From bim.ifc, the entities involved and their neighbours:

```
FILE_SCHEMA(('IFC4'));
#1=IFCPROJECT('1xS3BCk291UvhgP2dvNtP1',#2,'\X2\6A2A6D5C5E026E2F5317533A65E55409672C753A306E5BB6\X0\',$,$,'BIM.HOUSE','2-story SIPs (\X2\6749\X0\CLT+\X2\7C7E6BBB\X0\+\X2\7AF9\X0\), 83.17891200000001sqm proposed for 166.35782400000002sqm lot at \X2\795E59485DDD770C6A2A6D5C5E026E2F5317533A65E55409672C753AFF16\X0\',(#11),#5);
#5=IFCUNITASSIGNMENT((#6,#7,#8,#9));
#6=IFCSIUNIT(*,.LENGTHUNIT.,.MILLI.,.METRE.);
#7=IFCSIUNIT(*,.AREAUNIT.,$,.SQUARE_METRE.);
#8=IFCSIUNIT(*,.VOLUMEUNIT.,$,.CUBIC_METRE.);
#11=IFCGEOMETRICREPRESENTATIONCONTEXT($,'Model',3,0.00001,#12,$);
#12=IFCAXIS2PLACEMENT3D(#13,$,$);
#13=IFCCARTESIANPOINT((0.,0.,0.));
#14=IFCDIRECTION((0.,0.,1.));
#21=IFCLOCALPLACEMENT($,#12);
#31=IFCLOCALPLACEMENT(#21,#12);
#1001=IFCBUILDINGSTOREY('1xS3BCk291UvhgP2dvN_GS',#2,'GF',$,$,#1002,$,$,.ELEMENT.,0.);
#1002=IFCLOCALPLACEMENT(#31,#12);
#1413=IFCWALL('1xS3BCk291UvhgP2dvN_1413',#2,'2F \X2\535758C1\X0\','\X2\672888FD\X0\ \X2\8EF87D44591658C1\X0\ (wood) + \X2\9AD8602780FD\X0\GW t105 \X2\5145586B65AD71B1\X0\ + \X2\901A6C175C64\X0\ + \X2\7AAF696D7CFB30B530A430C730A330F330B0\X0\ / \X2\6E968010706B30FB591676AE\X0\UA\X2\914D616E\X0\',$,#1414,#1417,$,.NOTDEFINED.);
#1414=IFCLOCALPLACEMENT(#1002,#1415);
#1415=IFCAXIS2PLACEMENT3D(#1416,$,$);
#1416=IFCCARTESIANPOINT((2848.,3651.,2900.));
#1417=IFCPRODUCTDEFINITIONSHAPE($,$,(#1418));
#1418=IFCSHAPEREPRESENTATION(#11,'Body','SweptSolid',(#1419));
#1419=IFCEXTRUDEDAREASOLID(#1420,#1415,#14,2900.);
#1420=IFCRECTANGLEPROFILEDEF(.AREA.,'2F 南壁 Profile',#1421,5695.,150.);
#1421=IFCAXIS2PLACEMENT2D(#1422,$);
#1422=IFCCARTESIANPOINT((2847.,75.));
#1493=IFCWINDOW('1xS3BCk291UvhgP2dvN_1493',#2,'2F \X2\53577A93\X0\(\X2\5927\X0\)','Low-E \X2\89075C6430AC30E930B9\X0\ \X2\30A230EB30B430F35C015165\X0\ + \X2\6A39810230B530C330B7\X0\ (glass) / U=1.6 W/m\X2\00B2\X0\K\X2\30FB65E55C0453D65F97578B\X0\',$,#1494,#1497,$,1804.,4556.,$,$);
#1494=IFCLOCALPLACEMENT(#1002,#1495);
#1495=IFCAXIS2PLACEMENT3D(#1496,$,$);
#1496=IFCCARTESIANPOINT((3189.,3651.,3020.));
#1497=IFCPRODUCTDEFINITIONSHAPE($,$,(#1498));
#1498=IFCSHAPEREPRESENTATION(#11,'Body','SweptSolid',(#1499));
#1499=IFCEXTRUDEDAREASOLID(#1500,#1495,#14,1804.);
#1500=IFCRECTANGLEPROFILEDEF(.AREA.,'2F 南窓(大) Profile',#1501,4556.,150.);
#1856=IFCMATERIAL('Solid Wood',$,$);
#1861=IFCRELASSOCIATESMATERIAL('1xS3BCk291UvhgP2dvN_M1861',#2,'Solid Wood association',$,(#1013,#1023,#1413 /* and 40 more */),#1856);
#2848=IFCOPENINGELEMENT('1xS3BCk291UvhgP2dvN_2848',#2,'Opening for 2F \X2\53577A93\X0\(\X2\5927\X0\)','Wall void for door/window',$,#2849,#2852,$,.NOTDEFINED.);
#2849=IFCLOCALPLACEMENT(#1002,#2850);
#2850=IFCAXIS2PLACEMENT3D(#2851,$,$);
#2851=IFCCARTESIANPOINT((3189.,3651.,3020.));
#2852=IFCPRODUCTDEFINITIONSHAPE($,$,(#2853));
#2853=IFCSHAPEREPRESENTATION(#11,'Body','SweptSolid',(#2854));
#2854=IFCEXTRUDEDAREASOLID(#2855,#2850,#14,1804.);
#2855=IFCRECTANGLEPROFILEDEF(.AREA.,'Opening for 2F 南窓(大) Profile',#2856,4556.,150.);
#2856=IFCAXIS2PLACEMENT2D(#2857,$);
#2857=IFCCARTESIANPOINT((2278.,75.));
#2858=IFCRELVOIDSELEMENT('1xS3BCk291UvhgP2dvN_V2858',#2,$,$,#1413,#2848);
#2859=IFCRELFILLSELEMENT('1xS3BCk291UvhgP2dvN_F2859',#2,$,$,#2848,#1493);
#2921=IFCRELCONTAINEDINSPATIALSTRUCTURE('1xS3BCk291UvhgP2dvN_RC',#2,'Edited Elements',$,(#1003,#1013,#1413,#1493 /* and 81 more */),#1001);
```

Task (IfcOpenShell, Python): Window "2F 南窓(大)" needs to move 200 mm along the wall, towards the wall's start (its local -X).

```python
import ifcopenshell
import ifcopenshell.api.geometry
import ifcopenshell.util.placement
import ifcopenshell.util.unit

model = ifcopenshell.open("bim.ifc")
unit_scale = ifcopenshell.util.unit.calculate_unit_scale(model)

window = model.by_guid("1xS3BCk291UvhgP2dvN_1493")
opening = window.FillsVoids[0].RelatingOpeningElement
wall = opening.VoidsElements[0].RelatingBuildingElement

wall_matrix = ifcopenshell.util.placement.get_local_placement(wall.ObjectPlacement)
shift = wall_matrix[:3, 0] * -0.2 / unit_scale
before = ifcopenshell.util.placement.get_local_placement(window.ObjectPlacement)[:3, 3].copy()

# The window is not placed relative to its opening, so move both.
for product in (opening, window):
    matrix = ifcopenshell.util.placement.get_local_placement(product.ObjectPlacement)
    matrix[:3, 3] += shift
    ifcopenshell.api.geometry.edit_object_placement(model, product=product, matrix=matrix, is_si=False)

after = ifcopenshell.util.placement.get_local_placement(window.ObjectPlacement)[:3, 3]
print("window moved by", (after - before).round(3) + 0.0)

model.write("bim_rev.ifc")
```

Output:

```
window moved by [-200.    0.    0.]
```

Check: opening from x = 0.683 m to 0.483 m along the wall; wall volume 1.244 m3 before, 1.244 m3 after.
